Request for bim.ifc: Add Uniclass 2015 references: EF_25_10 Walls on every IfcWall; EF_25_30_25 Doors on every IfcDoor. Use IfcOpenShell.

First a look at what the model holds.

```python
import ifcopenshell

model = ifcopenshell.open("bim.ifc")
print(model.schema)
print("classifications:", [c.Name for c in model.by_type("IfcClassification")])
for ifc_class in ("IfcDoor", "IfcRoof", "IfcStair", "IfcWall", "IfcWindow"):
    print(ifc_class, len(model.by_type(ifc_class)))
```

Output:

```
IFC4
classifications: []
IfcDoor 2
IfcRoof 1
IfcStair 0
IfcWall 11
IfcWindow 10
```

```python
import ifcopenshell
import ifcopenshell.api.classification

model = ifcopenshell.open("bim.ifc")

system = ifcopenshell.api.classification.add_classification(model, classification="Uniclass 2015")

codes = {
    "IfcWall": ("EF_25_10", "Walls"),
    "IfcDoor": ("EF_25_30_25", "Doors"),
}
for ifc_class, (code, name) in codes.items():
    products = model.by_type(ifc_class)
    ifcopenshell.api.classification.add_reference(
        model, products=products, classification=system, identification=code, name=name
    )
    print(code, len(products))

model.write("bim_rev.ifc")
```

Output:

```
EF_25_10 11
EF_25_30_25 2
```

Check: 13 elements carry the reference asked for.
